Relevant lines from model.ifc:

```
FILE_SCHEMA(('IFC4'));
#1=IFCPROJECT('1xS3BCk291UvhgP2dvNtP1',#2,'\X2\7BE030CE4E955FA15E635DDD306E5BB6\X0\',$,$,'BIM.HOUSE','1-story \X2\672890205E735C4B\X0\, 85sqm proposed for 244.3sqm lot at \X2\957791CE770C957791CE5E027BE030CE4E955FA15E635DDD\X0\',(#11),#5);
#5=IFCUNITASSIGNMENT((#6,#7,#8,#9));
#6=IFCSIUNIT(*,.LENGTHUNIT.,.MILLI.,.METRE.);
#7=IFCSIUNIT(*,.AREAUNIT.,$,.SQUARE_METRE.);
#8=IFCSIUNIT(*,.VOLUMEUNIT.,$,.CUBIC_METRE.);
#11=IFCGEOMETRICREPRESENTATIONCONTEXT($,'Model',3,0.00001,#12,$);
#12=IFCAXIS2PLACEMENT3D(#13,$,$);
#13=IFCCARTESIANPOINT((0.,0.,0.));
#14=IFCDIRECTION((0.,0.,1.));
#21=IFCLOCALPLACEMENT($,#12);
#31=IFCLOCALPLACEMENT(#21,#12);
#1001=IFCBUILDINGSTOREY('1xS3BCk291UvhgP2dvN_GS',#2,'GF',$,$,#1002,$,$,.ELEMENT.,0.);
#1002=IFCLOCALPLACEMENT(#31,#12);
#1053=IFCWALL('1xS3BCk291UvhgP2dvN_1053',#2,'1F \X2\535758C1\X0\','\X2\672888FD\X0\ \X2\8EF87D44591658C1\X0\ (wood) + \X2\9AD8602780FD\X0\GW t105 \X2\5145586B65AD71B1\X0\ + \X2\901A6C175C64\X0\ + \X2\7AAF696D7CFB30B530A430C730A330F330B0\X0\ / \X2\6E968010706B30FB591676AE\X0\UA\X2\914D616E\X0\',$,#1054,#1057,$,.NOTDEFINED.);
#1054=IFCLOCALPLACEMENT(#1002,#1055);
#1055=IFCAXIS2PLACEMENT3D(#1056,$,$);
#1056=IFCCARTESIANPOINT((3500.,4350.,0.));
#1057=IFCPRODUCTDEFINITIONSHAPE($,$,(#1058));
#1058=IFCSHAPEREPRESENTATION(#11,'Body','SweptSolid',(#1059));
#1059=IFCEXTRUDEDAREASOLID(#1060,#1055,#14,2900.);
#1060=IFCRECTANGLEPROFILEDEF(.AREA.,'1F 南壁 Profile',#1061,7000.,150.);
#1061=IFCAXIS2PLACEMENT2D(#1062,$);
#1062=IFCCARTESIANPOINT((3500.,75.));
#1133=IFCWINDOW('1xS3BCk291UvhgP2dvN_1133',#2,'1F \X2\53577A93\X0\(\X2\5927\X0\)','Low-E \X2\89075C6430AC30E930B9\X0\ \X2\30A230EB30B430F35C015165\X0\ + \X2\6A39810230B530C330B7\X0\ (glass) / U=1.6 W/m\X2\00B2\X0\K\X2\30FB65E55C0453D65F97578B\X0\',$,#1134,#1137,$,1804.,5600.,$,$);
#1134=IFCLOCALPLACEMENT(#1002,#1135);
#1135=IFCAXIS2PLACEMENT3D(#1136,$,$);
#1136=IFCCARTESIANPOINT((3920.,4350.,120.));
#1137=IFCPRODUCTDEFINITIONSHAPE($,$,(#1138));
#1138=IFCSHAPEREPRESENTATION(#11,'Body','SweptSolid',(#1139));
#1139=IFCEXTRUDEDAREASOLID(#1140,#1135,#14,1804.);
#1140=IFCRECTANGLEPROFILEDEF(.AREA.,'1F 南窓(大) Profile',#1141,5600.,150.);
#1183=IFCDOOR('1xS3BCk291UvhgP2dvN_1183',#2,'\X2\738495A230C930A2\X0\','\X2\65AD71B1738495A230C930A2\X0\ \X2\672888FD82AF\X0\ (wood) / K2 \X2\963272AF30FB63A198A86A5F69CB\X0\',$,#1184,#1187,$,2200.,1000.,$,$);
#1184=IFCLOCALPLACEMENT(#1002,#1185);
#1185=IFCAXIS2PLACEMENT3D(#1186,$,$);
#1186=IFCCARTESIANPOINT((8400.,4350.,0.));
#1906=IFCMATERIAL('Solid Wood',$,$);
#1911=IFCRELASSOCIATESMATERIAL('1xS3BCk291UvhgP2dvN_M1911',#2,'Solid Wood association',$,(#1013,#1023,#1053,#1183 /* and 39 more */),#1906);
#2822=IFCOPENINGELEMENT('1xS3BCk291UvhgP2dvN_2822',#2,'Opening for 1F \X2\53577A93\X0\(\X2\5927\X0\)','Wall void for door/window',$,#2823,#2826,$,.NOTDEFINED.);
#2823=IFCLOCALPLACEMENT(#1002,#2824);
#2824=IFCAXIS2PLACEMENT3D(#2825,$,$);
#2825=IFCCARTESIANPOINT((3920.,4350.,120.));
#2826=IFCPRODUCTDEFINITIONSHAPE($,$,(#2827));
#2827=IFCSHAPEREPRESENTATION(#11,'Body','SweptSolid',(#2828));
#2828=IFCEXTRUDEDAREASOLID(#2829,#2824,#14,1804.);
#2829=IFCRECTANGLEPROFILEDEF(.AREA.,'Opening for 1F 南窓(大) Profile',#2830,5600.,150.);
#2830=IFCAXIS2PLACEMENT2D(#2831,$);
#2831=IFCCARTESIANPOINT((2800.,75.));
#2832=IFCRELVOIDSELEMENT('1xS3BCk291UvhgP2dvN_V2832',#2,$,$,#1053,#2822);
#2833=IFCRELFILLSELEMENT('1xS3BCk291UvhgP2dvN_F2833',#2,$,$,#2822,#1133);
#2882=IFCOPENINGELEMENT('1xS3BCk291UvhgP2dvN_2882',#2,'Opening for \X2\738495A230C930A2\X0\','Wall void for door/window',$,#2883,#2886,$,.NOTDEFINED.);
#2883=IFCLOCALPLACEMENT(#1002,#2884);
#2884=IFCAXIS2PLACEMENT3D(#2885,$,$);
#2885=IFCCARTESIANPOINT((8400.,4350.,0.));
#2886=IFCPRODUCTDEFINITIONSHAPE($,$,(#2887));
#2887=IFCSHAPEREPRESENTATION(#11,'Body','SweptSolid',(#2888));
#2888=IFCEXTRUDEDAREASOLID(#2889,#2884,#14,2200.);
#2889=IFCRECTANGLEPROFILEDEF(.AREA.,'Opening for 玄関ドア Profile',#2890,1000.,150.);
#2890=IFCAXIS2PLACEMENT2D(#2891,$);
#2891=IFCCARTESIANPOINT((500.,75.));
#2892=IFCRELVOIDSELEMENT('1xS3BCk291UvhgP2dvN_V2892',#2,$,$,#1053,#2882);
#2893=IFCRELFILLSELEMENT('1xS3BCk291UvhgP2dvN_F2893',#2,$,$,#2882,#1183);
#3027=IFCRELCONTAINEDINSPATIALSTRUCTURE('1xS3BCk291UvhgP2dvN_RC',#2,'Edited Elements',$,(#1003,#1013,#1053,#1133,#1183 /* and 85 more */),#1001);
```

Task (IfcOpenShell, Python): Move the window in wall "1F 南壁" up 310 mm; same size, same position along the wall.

```python
import numpy as np
import ifcopenshell
import ifcopenshell.api.geometry
import ifcopenshell.util.placement
import ifcopenshell.util.unit

model = ifcopenshell.open("model.ifc")
unit_scale = ifcopenshell.util.unit.calculate_unit_scale(model)

window = model.by_id(1133)
opening = window.FillsVoids[0].RelatingOpeningElement
dz = 0.31 / unit_scale

shift = np.array([0.0, 0.0, dz])
# The window is not placed relative to its opening, so move both.
for product in (opening, window):
    matrix = ifcopenshell.util.placement.get_local_placement(product.ObjectPlacement)
    matrix[:3, 3] += shift
    ifcopenshell.api.geometry.edit_object_placement(model, product=product, matrix=matrix, is_si=False)

print(f"moved by {dz * unit_scale:+.3f} m")

model.write("model_rev.ifc")
```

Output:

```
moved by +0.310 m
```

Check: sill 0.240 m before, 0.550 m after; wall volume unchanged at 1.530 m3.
